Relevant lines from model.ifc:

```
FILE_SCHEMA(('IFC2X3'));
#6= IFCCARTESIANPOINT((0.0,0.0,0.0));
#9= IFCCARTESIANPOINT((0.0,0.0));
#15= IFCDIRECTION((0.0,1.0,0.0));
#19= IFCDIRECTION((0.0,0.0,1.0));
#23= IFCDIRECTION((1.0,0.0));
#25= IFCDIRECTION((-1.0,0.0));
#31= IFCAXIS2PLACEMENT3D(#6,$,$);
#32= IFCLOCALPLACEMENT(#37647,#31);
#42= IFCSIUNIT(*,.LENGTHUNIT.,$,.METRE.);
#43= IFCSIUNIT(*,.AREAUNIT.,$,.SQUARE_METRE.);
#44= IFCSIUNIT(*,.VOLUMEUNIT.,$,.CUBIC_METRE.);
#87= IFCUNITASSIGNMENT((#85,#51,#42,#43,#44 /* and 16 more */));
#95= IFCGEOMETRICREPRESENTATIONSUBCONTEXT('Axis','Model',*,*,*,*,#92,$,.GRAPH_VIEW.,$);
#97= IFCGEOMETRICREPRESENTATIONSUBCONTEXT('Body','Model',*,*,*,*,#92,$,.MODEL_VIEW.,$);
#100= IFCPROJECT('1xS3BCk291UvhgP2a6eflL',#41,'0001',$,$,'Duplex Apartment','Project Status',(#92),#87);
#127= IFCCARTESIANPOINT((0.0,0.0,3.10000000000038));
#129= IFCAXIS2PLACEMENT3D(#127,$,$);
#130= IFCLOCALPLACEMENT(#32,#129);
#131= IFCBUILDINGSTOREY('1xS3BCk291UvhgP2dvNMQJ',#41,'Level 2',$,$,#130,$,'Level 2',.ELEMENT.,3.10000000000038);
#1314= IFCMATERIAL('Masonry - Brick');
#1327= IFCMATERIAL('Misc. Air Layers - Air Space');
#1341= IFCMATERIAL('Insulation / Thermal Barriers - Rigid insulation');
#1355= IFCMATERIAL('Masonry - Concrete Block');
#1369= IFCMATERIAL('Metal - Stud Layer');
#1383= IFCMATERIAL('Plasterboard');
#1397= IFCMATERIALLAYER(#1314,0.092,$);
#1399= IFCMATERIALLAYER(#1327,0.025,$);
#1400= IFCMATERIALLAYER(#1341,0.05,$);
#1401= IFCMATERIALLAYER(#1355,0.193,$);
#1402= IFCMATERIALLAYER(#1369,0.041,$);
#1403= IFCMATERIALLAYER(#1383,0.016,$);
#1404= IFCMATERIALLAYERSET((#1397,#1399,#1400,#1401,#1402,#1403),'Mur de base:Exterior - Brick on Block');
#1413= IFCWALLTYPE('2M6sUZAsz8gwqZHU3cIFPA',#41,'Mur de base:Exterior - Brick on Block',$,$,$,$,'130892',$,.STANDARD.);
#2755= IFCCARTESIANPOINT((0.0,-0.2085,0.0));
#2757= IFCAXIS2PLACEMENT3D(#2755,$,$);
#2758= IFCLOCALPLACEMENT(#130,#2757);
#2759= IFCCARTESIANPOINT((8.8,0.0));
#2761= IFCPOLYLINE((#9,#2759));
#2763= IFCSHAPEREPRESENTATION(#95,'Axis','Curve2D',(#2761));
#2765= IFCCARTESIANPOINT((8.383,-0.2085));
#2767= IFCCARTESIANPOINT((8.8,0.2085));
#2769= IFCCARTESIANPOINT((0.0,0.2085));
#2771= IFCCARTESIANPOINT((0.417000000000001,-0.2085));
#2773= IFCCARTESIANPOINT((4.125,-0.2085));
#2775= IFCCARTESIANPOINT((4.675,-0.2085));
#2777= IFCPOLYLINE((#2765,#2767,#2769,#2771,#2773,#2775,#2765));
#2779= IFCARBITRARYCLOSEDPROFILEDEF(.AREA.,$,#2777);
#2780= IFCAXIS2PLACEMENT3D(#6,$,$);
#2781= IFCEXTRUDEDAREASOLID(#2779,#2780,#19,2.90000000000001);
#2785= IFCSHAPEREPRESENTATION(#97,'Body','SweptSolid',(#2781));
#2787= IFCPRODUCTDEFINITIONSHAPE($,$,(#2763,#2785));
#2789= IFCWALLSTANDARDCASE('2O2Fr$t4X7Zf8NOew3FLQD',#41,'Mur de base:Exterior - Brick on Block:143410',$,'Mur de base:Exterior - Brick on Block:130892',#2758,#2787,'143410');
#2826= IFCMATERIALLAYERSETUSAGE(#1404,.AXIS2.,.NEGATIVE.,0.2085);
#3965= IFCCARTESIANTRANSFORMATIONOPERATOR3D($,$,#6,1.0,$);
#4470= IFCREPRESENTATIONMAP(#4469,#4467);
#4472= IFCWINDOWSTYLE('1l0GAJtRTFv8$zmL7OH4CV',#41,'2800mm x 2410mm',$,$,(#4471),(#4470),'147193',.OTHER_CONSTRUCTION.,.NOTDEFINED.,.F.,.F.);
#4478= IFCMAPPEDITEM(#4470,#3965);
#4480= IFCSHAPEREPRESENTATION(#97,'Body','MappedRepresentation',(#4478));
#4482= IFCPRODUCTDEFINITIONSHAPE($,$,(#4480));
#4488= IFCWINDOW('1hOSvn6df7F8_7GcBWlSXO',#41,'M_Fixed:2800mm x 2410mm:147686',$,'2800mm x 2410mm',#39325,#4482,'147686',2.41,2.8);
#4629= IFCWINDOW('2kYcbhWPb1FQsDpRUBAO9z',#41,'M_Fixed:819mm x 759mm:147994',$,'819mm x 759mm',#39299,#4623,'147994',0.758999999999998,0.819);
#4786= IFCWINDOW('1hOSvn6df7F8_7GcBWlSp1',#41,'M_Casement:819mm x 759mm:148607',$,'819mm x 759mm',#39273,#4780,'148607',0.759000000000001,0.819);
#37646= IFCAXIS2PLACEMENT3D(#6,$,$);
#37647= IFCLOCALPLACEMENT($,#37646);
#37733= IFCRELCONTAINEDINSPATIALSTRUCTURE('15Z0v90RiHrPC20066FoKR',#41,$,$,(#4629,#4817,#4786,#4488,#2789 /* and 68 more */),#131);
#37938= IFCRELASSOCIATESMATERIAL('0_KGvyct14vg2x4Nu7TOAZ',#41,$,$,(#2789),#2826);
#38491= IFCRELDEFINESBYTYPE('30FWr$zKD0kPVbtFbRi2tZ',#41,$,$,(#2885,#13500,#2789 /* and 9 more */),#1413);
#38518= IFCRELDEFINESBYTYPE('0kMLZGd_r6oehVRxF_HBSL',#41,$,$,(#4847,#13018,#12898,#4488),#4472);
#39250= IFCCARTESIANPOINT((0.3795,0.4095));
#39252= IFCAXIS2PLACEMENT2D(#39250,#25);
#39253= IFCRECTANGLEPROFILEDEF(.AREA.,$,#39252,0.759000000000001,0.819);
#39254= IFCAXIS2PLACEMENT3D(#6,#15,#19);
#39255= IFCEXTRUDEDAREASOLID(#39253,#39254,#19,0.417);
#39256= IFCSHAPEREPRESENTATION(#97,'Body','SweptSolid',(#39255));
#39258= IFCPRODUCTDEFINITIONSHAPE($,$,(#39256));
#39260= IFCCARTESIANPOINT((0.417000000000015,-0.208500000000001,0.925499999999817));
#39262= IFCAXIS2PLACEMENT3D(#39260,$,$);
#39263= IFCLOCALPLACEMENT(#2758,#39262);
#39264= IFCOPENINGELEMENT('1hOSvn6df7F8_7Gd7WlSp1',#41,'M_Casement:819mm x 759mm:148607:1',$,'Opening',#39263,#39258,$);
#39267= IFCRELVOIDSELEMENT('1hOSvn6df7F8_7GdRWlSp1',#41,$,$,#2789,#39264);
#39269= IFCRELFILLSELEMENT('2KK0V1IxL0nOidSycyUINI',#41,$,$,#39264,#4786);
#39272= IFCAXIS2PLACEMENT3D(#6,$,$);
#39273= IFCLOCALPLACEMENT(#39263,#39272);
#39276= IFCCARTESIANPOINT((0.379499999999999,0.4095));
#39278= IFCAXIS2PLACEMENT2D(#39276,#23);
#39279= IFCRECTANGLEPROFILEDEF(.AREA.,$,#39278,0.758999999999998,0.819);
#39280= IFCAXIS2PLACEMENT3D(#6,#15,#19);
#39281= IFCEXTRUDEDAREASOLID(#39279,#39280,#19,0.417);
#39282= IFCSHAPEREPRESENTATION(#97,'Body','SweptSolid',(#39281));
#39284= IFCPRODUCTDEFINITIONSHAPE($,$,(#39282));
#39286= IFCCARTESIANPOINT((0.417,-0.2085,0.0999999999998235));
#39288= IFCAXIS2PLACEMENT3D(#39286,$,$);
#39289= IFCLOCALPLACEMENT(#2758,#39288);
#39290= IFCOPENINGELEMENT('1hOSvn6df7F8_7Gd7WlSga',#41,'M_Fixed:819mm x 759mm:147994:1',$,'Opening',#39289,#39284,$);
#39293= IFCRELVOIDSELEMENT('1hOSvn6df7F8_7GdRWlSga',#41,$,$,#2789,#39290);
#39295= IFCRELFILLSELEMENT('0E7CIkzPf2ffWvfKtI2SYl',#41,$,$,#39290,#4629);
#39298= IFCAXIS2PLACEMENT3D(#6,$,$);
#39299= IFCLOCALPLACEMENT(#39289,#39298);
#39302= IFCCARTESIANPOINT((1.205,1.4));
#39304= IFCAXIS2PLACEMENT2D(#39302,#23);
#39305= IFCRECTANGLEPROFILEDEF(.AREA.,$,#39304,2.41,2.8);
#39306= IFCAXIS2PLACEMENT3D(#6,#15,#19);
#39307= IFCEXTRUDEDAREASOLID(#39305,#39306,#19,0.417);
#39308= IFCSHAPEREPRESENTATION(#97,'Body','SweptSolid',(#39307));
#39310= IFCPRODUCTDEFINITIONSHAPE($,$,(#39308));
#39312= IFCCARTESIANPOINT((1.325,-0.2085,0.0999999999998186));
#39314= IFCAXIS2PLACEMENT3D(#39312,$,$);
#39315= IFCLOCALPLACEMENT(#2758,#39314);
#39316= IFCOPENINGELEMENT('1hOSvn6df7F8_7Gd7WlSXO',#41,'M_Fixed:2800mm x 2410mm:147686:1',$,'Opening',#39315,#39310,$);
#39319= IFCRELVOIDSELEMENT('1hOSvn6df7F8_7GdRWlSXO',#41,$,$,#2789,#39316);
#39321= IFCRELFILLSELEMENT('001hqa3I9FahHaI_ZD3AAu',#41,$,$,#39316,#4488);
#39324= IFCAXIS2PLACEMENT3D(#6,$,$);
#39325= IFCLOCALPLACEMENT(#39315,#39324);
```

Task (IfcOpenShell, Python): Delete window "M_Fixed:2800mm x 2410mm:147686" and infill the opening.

```python
import ifcopenshell
import ifcopenshell.api.feature
import ifcopenshell.api.root
import ifcopenshell.geom
import ifcopenshell.util.shape

model = ifcopenshell.open("model.ifc")
settings = ifcopenshell.geom.settings()


def volume(element):
    """Net volume in cubic metres, openings subtracted."""
    shape = ifcopenshell.geom.create_shape(settings, element)
    return ifcopenshell.util.shape.get_volume(shape.geometry)


window = model.by_id(4488)
opening = window.FillsVoids[0].RelatingOpeningElement
wall = opening.VoidsElements[0].RelatingBuildingElement
before = volume(wall)

ifcopenshell.api.root.remove_product(model, product=window)
ifcopenshell.api.feature.remove_feature(model, feature=opening)

after = volume(wall)

print(f"wall volume {before:.3f} -> {after:.3f} m3")

model.write("model-out.ifc")
```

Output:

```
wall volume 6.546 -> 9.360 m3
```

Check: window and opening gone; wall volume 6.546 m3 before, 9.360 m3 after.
